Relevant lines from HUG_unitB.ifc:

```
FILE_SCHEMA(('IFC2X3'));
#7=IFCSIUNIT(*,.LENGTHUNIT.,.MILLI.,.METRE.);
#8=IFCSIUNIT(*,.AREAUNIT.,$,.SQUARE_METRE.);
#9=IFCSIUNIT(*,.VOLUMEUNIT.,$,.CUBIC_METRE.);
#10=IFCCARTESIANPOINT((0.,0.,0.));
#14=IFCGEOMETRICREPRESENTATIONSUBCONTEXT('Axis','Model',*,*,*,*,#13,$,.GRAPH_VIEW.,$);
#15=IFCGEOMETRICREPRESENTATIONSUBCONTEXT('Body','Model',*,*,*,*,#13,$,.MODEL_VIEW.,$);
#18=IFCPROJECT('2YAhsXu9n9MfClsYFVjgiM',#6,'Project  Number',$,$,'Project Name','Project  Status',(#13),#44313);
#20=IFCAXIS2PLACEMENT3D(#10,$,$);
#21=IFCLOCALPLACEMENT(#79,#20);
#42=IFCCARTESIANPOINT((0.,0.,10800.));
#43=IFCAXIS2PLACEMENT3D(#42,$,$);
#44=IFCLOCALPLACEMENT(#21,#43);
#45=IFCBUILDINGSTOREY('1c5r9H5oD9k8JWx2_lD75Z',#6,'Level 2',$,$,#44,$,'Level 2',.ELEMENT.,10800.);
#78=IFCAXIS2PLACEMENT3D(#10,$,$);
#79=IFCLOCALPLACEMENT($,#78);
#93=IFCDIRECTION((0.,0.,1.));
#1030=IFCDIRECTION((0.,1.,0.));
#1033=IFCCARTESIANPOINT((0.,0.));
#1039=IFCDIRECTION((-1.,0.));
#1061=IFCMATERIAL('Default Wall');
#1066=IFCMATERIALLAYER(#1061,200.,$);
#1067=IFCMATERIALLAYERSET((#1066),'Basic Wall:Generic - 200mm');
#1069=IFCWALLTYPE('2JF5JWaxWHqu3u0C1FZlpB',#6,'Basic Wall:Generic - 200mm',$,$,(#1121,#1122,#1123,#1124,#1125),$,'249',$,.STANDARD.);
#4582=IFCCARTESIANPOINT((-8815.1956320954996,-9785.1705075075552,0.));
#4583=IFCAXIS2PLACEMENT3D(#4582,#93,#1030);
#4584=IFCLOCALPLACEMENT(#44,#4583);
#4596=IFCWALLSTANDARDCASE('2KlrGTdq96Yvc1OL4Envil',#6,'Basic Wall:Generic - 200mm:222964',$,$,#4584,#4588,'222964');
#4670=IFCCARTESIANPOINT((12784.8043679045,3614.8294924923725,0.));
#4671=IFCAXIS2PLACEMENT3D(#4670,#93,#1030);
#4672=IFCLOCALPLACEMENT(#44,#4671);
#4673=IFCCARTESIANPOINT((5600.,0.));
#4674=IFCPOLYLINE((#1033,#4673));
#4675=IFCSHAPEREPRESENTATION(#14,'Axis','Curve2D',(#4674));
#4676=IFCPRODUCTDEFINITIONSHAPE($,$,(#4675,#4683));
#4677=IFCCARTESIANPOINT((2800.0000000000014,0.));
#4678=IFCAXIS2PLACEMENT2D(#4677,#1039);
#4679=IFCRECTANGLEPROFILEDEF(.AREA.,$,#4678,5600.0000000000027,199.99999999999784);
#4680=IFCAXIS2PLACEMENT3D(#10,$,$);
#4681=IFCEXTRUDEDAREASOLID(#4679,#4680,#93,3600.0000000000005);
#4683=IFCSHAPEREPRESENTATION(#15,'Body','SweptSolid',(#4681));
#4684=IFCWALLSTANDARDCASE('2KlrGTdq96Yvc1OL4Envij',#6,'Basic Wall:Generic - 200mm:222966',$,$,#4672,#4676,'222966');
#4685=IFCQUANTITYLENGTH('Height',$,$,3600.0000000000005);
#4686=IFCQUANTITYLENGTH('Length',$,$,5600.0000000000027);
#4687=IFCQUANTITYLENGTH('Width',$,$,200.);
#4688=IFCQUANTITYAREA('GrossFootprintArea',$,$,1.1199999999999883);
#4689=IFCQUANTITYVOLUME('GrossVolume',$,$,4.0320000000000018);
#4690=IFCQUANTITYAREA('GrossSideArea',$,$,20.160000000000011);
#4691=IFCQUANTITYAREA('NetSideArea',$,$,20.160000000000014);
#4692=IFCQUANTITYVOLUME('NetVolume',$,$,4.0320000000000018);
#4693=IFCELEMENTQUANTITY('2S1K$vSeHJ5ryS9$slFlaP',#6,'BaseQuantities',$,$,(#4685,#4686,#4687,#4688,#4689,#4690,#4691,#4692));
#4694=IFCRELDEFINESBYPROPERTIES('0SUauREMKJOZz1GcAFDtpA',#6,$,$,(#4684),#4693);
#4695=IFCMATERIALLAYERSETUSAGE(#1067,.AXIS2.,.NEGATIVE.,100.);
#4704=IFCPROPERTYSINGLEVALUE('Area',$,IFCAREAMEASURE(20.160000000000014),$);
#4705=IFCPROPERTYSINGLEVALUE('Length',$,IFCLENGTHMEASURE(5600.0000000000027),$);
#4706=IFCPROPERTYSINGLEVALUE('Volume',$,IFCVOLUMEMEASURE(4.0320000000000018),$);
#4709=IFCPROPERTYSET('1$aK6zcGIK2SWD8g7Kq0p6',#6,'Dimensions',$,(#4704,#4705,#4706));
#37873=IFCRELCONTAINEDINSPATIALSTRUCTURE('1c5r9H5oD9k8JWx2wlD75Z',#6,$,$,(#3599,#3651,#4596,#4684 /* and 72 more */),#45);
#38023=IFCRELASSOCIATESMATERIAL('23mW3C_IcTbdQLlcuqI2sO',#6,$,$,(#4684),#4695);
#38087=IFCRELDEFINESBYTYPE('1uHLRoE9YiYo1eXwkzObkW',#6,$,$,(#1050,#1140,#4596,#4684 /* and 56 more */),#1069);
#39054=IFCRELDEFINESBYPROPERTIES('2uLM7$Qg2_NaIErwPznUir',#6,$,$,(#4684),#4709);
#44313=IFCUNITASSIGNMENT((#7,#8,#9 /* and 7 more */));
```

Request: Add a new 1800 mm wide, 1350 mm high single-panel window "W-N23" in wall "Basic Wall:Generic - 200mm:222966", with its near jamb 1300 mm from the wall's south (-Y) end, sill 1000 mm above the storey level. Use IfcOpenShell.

```python
import numpy as np
import ifcopenshell
import ifcopenshell.api.feature
import ifcopenshell.api.geometry
import ifcopenshell.api.pset
import ifcopenshell.api.root
import ifcopenshell.api.spatial
import ifcopenshell.api.type
import ifcopenshell.geom
import ifcopenshell.util.element
import ifcopenshell.util.placement
import ifcopenshell.util.representation
import ifcopenshell.util.shape
import ifcopenshell.util.unit

model = ifcopenshell.open("HUG_unitB.ifc")
unit_scale = ifcopenshell.util.unit.calculate_unit_scale(model)
area_scale = ifcopenshell.util.unit.calculate_unit_scale(model, "AREAUNIT")
volume_scale = ifcopenshell.util.unit.calculate_unit_scale(model, "VOLUMEUNIT")
settings = ifcopenshell.geom.settings()


def volume(element):
    """Net volume in cubic metres, openings subtracted."""
    shape = ifcopenshell.geom.create_shape(settings, element)
    return ifcopenshell.util.shape.get_volume(shape.geometry)


wall = model.by_guid("2KlrGTdq96Yvc1OL4Envij")
storey = ifcopenshell.util.element.get_container(wall, ifc_class="IfcBuildingStorey")
context = ifcopenshell.util.representation.get_context(model, "Model", "Body", "MODEL_VIEW")
before = volume(wall)

width, height, from_end, sill = 1.8, 1.35, 1.3, 1  # metres

# The wall runs along its own X axis, and the end named is its -X end.
wall_shape = ifcopenshell.geom.create_shape(settings, wall)
x, y, z = ifcopenshell.util.shape.get_vertices(wall_shape.geometry).T
start = x.min() + from_end
face, thickness = float(y.min()), float(y.max() - y.min())
wall_matrix = ifcopenshell.util.placement.get_local_placement(wall.ObjectPlacement)
level = ifcopenshell.util.placement.get_local_placement(storey.ObjectPlacement)[2, 3]


def in_wall(x, y):
    """Placement at x, y metres in the wall's axes, at sill height."""
    matrix = wall_matrix.copy()
    matrix[:, 3] = wall_matrix @ np.array([x / unit_scale, y / unit_scale, 0.0, 1.0])
    matrix[2, 3] = level + sill / unit_scale
    return matrix


# Opening: a box that overshoots both wall faces by 50 mm.
opening = ifcopenshell.api.root.create_entity(model, ifc_class="IfcOpeningElement")
box = ifcopenshell.api.geometry.add_wall_representation(
    model, context=context, length=width, height=height, thickness=thickness + 0.1
)
ifcopenshell.api.geometry.assign_representation(model, product=opening, representation=box)
ifcopenshell.api.geometry.edit_object_placement(model, product=opening, matrix=in_wall(start, face - 0.05), is_si=False)
ifcopenshell.api.feature.add_feature(model, feature=opening, element=wall)

window = ifcopenshell.api.root.create_entity(model, ifc_class="IfcWindow", name="W-N23")
window.OverallWidth, window.OverallHeight = width / unit_scale, height / unit_scale
body = ifcopenshell.api.geometry.add_window_representation(
    model,
    context=context,
    overall_width=window.OverallWidth,
    overall_height=window.OverallHeight,
    partition_type="SINGLE_PANEL",
)
ifcopenshell.api.geometry.assign_representation(model, product=window, representation=body)
ifcopenshell.api.spatial.assign_container(model, products=[window], relating_structure=storey)
fills = ifcopenshell.api.feature.add_filling(model, opening=opening, element=window)
fills.OwnerHistory = window.OwnerHistory  # required in IFC2X3

# IFC2X3 keeps the operation on the window style.
style = ifcopenshell.api.root.create_entity(model, ifc_class="IfcWindowStyle", name="W-N23")
style.OperationType, style.ConstructionType = "SINGLE_PANEL", "NOTDEFINED"
style.ParameterTakesPrecedence = style.Sizeable = False
ifcopenshell.api.type.assign_type(model, related_objects=[window], relating_type=style)

# Centre the window in the wall's thickness.
ifcopenshell.api.geometry.edit_object_placement(model, product=window, matrix=in_wall(start, face), is_si=False)
window_shape = ifcopenshell.geom.create_shape(settings, window)
depth = ifcopenshell.util.shape.get_vertices(window_shape.geometry)[:, 1]
offset = face + thickness / 2 - (depth.min() + depth.max()) / 2
ifcopenshell.api.geometry.edit_object_placement(model, product=window, matrix=in_wall(start, offset), is_si=False)

after = volume(wall)

# Update the wall's stored quantities.
qto = model.by_id(ifcopenshell.util.element.get_pset(wall, "BaseQuantities", should_inherit=False)["id"])
ifcopenshell.api.pset.edit_qto(model, qto=qto, properties={
    "NetSideArea": after / thickness / area_scale,
    "NetVolume": after / volume_scale,
})
pset = model.by_id(ifcopenshell.util.element.get_pset(wall, "Dimensions", should_inherit=False)["id"])
ifcopenshell.api.pset.edit_pset(model, pset=pset, properties={
    "Area": model.create_entity("IfcAreaMeasure", after / thickness / area_scale),
    "Volume": model.create_entity("IfcVolumeMeasure", after / volume_scale),
})

print(f"wall volume {before:.3f} -> {after:.3f} m3")

model.write("HUG_unitB_rev.ifc")
```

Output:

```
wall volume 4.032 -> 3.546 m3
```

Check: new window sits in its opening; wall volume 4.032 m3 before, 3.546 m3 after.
